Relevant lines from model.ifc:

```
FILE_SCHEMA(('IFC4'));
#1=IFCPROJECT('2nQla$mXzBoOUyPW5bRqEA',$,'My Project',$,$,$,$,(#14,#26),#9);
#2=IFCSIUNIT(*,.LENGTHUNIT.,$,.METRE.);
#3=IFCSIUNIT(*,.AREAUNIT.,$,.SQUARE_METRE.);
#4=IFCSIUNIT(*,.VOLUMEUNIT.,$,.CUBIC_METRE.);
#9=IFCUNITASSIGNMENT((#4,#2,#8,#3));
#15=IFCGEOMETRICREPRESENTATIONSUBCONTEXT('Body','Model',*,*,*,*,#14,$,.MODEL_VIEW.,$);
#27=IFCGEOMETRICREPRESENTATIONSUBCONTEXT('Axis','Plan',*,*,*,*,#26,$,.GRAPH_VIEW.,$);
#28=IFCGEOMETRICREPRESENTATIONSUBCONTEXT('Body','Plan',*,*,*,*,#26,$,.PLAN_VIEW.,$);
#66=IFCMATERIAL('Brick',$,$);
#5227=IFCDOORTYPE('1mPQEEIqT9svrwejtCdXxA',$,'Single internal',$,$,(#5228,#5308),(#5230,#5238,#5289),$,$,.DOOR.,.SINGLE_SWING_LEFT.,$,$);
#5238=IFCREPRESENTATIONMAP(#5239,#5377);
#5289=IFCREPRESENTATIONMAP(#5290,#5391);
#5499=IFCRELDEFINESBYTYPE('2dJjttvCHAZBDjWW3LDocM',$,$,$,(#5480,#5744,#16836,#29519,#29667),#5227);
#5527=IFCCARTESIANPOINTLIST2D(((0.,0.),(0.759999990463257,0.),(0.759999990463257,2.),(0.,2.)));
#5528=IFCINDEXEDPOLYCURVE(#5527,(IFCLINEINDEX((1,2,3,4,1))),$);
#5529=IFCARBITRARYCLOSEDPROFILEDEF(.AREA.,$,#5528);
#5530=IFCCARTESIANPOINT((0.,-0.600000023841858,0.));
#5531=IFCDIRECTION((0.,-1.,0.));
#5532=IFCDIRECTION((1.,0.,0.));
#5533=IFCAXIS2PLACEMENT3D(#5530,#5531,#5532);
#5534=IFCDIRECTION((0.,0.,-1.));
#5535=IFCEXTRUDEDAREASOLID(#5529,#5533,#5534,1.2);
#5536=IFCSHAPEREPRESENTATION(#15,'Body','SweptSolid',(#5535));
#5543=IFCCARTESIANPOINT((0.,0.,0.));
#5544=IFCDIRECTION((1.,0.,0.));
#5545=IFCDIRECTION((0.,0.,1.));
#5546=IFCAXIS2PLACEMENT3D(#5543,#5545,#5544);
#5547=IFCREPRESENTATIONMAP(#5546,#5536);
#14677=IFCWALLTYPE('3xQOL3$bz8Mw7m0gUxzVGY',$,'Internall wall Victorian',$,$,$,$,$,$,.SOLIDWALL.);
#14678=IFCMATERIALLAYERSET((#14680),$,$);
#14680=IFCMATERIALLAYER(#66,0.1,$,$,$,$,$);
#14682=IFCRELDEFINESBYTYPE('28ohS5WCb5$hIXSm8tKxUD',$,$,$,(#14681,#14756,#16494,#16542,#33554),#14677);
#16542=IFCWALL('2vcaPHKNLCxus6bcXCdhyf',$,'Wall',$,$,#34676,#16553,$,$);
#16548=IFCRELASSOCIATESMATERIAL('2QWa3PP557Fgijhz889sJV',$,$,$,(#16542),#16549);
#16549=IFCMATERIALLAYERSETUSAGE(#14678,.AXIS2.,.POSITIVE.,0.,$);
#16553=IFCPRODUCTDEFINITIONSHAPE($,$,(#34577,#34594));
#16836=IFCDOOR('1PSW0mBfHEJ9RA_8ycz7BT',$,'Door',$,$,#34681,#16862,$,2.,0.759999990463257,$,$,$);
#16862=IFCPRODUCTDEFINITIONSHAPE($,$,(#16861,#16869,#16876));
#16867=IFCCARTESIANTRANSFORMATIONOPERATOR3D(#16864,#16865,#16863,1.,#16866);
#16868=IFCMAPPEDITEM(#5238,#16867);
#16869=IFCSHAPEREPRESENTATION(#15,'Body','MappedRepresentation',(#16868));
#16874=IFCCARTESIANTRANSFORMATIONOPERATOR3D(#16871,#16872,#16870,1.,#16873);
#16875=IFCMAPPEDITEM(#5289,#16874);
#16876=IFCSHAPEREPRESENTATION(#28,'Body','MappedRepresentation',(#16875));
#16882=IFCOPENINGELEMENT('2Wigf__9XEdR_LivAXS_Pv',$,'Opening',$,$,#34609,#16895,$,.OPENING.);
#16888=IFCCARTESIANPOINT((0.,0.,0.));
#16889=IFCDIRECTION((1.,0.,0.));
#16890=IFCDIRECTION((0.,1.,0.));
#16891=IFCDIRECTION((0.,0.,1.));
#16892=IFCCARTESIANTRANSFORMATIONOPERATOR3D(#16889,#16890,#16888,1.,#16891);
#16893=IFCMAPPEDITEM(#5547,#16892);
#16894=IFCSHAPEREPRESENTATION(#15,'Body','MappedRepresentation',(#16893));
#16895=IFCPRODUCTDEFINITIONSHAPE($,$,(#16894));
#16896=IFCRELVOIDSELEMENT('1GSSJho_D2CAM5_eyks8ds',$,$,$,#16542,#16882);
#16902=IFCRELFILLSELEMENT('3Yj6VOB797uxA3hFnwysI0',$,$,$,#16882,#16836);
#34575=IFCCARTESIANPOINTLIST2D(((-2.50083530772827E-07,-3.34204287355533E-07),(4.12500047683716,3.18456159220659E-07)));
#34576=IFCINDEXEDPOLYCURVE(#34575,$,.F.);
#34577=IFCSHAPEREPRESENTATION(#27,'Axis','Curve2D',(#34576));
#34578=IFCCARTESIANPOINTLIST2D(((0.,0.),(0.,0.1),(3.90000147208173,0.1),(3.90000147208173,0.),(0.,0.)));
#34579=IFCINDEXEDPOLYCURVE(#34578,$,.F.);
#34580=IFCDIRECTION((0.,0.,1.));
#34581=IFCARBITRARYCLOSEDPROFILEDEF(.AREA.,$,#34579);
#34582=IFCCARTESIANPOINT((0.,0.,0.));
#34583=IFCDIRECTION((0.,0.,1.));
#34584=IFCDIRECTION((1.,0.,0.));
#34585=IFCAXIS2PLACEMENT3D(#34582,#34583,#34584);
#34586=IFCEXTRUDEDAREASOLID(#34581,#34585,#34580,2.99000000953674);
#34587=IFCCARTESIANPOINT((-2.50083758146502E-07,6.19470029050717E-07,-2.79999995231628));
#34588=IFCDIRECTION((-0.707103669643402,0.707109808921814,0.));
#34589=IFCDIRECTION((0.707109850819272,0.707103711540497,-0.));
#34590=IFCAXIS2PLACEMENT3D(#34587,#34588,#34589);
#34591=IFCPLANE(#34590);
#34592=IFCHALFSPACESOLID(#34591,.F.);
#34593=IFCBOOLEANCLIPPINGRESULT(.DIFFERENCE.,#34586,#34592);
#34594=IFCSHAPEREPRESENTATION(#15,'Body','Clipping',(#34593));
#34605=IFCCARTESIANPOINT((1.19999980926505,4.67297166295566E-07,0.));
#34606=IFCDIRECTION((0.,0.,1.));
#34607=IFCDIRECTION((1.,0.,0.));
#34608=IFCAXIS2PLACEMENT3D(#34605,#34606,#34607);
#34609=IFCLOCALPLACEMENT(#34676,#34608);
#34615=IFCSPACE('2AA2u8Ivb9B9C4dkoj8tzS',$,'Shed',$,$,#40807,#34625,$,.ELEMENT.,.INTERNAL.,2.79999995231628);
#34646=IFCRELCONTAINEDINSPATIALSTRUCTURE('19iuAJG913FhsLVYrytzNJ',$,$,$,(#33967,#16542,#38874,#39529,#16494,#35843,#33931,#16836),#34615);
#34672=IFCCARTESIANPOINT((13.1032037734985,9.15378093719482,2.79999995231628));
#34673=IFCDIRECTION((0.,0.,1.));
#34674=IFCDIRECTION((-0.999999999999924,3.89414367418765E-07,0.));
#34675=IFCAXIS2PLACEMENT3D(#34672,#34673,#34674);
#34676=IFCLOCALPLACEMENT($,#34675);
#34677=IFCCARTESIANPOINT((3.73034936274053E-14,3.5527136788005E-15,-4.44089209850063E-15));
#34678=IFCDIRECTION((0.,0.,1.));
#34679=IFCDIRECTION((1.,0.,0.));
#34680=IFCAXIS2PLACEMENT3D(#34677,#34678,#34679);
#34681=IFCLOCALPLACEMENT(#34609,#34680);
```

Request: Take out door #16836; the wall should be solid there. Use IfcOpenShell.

```python
import ifcopenshell
import ifcopenshell.api.feature
import ifcopenshell.api.root
import ifcopenshell.geom
import ifcopenshell.util.shape

model = ifcopenshell.open("model.ifc")
settings = ifcopenshell.geom.settings()


def volume(element):
    """Net volume in cubic metres, openings subtracted."""
    shape = ifcopenshell.geom.create_shape(settings, element)
    return ifcopenshell.util.shape.get_volume(shape.geometry)


door = model.by_id(16836)
opening = door.FillsVoids[0].RelatingOpeningElement
wall = opening.VoidsElements[0].RelatingBuildingElement
before = volume(wall)

ifcopenshell.api.root.remove_product(model, product=door)
ifcopenshell.api.feature.remove_feature(model, feature=opening)

after = volume(wall)

print(f"wall volume {before:.3f} -> {after:.3f} m3")

model.write("model_rev.ifc")
```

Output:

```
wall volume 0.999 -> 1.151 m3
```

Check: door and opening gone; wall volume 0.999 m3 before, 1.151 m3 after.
